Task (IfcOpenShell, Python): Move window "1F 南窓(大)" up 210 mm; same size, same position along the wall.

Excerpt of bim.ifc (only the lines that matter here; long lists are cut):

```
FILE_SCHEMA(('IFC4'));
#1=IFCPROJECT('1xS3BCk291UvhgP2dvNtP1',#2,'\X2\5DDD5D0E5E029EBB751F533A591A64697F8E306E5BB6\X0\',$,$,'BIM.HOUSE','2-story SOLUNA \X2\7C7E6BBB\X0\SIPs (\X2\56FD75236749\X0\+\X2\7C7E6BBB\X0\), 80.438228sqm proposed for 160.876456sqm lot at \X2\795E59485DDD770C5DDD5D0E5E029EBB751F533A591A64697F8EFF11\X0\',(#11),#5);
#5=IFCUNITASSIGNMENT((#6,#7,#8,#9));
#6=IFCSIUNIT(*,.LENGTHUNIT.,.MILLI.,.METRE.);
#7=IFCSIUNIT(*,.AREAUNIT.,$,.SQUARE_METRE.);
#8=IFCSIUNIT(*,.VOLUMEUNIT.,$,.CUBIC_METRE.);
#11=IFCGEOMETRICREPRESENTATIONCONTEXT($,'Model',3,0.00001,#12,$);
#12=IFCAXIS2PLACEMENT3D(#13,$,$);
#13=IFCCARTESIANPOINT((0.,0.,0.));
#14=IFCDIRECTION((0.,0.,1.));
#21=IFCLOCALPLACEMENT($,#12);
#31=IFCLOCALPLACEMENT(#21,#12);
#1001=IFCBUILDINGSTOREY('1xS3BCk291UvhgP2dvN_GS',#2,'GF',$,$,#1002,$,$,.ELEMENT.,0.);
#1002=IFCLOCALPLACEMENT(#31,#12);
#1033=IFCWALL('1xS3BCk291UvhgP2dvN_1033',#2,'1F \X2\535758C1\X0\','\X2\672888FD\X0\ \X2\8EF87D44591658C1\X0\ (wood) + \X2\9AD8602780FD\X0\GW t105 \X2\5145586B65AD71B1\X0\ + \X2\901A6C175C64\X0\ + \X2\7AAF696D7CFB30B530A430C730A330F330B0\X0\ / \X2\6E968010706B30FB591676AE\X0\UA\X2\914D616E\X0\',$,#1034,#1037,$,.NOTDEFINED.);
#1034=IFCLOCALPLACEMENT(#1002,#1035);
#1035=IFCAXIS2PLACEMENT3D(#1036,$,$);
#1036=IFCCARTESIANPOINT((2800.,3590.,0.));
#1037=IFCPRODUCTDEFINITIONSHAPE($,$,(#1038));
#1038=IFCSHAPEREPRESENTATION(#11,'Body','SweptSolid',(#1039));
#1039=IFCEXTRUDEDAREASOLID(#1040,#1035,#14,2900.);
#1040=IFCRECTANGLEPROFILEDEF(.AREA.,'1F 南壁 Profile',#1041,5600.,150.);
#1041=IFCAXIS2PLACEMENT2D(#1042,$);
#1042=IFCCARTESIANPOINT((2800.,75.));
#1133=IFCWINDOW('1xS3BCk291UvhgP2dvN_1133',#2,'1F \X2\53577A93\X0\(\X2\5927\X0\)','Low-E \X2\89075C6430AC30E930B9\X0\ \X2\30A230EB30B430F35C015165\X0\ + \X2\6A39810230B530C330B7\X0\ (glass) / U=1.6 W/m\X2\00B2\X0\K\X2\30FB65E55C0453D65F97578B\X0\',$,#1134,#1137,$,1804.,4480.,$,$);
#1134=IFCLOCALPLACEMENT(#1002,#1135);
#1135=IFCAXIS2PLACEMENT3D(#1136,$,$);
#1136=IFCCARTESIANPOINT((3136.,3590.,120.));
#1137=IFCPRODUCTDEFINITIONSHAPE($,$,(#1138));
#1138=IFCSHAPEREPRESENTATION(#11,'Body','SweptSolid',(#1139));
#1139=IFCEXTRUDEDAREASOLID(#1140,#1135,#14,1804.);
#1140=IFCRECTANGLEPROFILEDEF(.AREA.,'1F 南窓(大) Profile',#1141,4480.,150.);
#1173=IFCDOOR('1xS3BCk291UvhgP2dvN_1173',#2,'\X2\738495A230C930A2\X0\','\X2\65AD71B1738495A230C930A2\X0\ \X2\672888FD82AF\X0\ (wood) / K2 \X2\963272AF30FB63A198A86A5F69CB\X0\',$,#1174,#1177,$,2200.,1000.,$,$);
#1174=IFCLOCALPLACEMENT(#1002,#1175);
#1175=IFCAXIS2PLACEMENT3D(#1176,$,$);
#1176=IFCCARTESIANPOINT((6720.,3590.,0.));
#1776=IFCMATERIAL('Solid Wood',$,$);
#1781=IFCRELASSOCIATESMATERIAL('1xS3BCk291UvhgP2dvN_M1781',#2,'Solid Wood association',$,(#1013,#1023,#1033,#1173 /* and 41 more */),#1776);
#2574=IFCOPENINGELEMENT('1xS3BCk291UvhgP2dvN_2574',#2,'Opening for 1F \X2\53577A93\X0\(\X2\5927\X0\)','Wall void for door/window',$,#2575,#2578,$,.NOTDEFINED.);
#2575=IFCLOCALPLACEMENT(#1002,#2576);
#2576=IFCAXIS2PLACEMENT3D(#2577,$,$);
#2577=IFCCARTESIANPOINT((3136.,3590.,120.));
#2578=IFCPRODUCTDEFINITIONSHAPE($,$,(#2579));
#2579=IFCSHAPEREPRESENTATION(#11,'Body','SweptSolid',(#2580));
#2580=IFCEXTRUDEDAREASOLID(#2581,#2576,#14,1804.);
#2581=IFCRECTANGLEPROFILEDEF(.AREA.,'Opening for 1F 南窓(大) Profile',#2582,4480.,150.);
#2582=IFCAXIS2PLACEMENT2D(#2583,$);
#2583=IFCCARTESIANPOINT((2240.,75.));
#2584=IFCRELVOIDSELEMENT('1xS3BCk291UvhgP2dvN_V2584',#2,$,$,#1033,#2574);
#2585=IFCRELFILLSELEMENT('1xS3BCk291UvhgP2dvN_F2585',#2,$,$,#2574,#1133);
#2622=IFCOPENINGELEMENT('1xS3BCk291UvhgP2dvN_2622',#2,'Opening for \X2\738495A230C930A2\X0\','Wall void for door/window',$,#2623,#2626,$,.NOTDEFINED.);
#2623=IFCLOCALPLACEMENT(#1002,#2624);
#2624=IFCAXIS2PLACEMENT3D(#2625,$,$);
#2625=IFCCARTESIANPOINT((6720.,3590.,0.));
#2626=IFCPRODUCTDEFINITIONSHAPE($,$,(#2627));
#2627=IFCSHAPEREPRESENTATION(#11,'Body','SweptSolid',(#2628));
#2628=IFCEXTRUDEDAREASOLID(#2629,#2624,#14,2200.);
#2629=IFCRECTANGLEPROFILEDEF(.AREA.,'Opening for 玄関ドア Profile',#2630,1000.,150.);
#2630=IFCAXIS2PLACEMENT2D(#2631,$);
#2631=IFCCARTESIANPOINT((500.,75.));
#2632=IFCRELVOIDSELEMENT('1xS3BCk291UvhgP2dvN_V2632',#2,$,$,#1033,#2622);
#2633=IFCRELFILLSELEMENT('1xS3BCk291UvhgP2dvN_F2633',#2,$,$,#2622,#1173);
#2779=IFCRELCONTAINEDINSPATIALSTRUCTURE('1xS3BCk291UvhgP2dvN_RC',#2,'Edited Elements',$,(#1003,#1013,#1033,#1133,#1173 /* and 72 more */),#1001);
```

```python
import numpy as np
import ifcopenshell
import ifcopenshell.api.geometry
import ifcopenshell.util.placement
import ifcopenshell.util.unit

model = ifcopenshell.open("bim.ifc")
unit_scale = ifcopenshell.util.unit.calculate_unit_scale(model)

window = model.by_guid("1xS3BCk291UvhgP2dvN_1133")
opening = window.FillsVoids[0].RelatingOpeningElement
dz = 210.0

shift = np.array([0.0, 0.0, dz])
# The window is not placed relative to its opening, so move both.
for product in (opening, window):
    matrix = ifcopenshell.util.placement.get_local_placement(product.ObjectPlacement)
    matrix[:3, 3] += shift
    ifcopenshell.api.geometry.edit_object_placement(model, product=product, matrix=matrix, is_si=False)

print(f"moved by {dz * unit_scale:+.3f} m")

model.write("bim_updated.ifc")
```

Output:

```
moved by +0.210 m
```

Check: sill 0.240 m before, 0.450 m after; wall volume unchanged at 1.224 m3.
